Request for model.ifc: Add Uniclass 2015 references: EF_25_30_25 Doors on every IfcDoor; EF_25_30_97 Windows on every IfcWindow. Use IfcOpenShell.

First a look at what the model holds.

```python
import ifcopenshell

model = ifcopenshell.open("model.ifc")
print(model.schema)
print("classifications:", [c.Name for c in model.by_type("IfcClassification")])
for ifc_class in ("IfcDoor", "IfcRoof", "IfcStair", "IfcWall", "IfcWindow"):
    print(ifc_class, len(model.by_type(ifc_class)))
```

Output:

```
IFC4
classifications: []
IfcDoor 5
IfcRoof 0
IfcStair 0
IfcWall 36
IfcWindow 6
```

```python
import ifcopenshell
import ifcopenshell.api.classification

model = ifcopenshell.open("model.ifc")

system = ifcopenshell.api.classification.add_classification(model, classification="Uniclass 2015")

codes = {
    "IfcDoor": ("EF_25_30_25", "Doors"),
    "IfcWindow": ("EF_25_30_97", "Windows"),
}
for ifc_class, (code, name) in codes.items():
    products = model.by_type(ifc_class)
    ifcopenshell.api.classification.add_reference(
        model, products=products, classification=system, identification=code, name=name
    )
    print(code, len(products))

model.write("model_edited.ifc")
```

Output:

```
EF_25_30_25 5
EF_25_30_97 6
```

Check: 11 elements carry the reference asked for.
